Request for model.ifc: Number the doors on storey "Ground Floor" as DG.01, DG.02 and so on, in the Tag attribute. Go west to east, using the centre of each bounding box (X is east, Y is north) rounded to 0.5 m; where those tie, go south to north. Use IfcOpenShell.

First a look at what the model holds.

```python
import ifcopenshell
import ifcopenshell.util.element
import ifcopenshell.util.placement

model = ifcopenshell.open("model.ifc")
print(model.schema)
storey = next(s for s in model.by_type("IfcBuildingStorey") if s.Name == "Ground Floor")
doors = [e for e in ifcopenshell.util.element.get_decomposition(storey) if e.is_a("IfcDoor")]
for e in sorted(doors, key=lambda e: e.id()):
    origin = ifcopenshell.util.placement.get_local_placement(e.ObjectPlacement)[:3, 3]
    print(e.id(), e.Tag, e.Name, origin.round(2) + 0.0, sep=" | ")
```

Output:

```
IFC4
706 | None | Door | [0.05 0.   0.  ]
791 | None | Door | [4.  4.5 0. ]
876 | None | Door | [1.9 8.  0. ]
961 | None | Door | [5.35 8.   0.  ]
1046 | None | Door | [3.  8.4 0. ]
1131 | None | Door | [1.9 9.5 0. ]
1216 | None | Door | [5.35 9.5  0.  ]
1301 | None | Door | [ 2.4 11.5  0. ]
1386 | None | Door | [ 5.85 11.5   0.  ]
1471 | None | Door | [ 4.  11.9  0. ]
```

```python
import ifcopenshell
import ifcopenshell.geom
import ifcopenshell.util.element
import ifcopenshell.util.shape

model = ifcopenshell.open("model.ifc")
settings = ifcopenshell.geom.settings()
settings.set("use-world-coords", True)


def centre(element):
    shape = ifcopenshell.geom.create_shape(settings, element)
    return ifcopenshell.util.shape.get_bbox_centroid(shape.geometry)


storey = next(s for s in model.by_type("IfcBuildingStorey") if s.Name == "Ground Floor")
doors = [e for e in ifcopenshell.util.element.get_decomposition(storey) if e.is_a("IfcDoor")]

# Insertion points can sit at a corner or the storey origin, so sort by the geometry (in metres).
centres = {e: centre(e) for e in doors}
doors.sort(key=lambda e: (round(centres[e][0] / 0.5), centres[e][1]))

for i, e in enumerate(doors, start=1):
    number = f"DG.{i:02d}"
    e.Tag = number
    print(e.id(), number)

model.write("model_v2.ifc")
```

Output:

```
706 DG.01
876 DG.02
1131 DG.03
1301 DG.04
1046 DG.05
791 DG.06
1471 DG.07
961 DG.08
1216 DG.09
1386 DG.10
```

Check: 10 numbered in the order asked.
